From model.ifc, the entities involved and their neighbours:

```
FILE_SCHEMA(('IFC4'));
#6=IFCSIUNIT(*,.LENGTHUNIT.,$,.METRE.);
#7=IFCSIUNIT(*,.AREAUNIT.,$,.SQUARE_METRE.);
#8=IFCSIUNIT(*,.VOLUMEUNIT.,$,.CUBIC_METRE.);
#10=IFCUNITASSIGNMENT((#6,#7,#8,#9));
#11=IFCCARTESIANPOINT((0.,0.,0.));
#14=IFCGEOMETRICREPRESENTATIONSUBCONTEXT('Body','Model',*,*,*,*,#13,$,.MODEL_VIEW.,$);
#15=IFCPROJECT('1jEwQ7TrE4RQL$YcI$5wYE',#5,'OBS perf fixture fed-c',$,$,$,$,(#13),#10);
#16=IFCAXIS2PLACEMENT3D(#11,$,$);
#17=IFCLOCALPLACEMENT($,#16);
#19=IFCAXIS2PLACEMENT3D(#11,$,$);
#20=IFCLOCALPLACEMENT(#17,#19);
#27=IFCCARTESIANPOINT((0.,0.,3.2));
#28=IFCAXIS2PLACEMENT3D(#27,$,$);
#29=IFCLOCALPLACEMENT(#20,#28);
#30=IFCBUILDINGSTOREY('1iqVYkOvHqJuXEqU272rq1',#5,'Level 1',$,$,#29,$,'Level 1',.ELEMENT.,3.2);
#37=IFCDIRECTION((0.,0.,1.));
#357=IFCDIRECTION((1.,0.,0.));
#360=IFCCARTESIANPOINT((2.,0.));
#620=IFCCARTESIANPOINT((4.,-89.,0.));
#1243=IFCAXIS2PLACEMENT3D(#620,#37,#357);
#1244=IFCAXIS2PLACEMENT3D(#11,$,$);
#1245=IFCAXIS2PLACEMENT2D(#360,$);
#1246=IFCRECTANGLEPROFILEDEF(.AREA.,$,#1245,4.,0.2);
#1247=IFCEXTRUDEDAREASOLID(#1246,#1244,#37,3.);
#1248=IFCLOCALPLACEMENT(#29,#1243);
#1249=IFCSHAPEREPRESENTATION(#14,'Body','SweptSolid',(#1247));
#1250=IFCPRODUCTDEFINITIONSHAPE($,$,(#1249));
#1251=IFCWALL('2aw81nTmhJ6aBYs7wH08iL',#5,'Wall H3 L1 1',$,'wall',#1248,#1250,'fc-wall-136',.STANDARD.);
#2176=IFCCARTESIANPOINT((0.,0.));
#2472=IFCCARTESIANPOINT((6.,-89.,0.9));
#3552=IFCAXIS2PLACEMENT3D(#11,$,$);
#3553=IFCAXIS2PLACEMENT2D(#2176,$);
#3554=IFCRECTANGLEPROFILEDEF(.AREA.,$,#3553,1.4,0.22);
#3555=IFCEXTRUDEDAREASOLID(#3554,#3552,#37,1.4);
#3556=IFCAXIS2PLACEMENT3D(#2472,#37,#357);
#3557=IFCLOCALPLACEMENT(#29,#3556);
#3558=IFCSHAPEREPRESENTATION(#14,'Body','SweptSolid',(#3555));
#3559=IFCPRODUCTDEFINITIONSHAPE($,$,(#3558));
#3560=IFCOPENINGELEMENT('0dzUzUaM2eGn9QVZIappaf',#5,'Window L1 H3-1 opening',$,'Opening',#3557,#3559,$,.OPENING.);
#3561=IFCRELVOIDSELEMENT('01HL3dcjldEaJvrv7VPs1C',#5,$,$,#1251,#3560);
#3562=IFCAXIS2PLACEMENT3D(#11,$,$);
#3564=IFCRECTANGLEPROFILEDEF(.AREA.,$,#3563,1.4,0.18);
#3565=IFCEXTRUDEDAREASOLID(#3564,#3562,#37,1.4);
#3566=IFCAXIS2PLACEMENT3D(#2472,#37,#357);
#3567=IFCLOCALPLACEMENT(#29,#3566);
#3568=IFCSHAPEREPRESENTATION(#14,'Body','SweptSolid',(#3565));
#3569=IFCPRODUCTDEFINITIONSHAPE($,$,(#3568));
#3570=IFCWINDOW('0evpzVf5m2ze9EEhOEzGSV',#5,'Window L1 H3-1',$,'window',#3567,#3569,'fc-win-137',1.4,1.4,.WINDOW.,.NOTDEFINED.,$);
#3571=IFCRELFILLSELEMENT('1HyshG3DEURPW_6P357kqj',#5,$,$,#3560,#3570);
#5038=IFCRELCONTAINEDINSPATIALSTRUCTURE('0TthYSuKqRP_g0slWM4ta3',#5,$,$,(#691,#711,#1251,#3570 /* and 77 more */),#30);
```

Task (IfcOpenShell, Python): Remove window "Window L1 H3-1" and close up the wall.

```python
import ifcopenshell
import ifcopenshell.api.feature
import ifcopenshell.api.root
import ifcopenshell.geom
import ifcopenshell.util.shape

model = ifcopenshell.open("model.ifc")
settings = ifcopenshell.geom.settings()


def volume(element):
    """Net volume in cubic metres, openings subtracted."""
    shape = ifcopenshell.geom.create_shape(settings, element)
    return ifcopenshell.util.shape.get_volume(shape.geometry)


window = model.by_id(3570)
opening = window.FillsVoids[0].RelatingOpeningElement
wall = opening.VoidsElements[0].RelatingBuildingElement
before = volume(wall)

ifcopenshell.api.root.remove_product(model, product=window)
ifcopenshell.api.feature.remove_feature(model, feature=opening)

after = volume(wall)

print(f"wall volume {before:.3f} -> {after:.3f} m3")

model.write("model_updated.ifc")
```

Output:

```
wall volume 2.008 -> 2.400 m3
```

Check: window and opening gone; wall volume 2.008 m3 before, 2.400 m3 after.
